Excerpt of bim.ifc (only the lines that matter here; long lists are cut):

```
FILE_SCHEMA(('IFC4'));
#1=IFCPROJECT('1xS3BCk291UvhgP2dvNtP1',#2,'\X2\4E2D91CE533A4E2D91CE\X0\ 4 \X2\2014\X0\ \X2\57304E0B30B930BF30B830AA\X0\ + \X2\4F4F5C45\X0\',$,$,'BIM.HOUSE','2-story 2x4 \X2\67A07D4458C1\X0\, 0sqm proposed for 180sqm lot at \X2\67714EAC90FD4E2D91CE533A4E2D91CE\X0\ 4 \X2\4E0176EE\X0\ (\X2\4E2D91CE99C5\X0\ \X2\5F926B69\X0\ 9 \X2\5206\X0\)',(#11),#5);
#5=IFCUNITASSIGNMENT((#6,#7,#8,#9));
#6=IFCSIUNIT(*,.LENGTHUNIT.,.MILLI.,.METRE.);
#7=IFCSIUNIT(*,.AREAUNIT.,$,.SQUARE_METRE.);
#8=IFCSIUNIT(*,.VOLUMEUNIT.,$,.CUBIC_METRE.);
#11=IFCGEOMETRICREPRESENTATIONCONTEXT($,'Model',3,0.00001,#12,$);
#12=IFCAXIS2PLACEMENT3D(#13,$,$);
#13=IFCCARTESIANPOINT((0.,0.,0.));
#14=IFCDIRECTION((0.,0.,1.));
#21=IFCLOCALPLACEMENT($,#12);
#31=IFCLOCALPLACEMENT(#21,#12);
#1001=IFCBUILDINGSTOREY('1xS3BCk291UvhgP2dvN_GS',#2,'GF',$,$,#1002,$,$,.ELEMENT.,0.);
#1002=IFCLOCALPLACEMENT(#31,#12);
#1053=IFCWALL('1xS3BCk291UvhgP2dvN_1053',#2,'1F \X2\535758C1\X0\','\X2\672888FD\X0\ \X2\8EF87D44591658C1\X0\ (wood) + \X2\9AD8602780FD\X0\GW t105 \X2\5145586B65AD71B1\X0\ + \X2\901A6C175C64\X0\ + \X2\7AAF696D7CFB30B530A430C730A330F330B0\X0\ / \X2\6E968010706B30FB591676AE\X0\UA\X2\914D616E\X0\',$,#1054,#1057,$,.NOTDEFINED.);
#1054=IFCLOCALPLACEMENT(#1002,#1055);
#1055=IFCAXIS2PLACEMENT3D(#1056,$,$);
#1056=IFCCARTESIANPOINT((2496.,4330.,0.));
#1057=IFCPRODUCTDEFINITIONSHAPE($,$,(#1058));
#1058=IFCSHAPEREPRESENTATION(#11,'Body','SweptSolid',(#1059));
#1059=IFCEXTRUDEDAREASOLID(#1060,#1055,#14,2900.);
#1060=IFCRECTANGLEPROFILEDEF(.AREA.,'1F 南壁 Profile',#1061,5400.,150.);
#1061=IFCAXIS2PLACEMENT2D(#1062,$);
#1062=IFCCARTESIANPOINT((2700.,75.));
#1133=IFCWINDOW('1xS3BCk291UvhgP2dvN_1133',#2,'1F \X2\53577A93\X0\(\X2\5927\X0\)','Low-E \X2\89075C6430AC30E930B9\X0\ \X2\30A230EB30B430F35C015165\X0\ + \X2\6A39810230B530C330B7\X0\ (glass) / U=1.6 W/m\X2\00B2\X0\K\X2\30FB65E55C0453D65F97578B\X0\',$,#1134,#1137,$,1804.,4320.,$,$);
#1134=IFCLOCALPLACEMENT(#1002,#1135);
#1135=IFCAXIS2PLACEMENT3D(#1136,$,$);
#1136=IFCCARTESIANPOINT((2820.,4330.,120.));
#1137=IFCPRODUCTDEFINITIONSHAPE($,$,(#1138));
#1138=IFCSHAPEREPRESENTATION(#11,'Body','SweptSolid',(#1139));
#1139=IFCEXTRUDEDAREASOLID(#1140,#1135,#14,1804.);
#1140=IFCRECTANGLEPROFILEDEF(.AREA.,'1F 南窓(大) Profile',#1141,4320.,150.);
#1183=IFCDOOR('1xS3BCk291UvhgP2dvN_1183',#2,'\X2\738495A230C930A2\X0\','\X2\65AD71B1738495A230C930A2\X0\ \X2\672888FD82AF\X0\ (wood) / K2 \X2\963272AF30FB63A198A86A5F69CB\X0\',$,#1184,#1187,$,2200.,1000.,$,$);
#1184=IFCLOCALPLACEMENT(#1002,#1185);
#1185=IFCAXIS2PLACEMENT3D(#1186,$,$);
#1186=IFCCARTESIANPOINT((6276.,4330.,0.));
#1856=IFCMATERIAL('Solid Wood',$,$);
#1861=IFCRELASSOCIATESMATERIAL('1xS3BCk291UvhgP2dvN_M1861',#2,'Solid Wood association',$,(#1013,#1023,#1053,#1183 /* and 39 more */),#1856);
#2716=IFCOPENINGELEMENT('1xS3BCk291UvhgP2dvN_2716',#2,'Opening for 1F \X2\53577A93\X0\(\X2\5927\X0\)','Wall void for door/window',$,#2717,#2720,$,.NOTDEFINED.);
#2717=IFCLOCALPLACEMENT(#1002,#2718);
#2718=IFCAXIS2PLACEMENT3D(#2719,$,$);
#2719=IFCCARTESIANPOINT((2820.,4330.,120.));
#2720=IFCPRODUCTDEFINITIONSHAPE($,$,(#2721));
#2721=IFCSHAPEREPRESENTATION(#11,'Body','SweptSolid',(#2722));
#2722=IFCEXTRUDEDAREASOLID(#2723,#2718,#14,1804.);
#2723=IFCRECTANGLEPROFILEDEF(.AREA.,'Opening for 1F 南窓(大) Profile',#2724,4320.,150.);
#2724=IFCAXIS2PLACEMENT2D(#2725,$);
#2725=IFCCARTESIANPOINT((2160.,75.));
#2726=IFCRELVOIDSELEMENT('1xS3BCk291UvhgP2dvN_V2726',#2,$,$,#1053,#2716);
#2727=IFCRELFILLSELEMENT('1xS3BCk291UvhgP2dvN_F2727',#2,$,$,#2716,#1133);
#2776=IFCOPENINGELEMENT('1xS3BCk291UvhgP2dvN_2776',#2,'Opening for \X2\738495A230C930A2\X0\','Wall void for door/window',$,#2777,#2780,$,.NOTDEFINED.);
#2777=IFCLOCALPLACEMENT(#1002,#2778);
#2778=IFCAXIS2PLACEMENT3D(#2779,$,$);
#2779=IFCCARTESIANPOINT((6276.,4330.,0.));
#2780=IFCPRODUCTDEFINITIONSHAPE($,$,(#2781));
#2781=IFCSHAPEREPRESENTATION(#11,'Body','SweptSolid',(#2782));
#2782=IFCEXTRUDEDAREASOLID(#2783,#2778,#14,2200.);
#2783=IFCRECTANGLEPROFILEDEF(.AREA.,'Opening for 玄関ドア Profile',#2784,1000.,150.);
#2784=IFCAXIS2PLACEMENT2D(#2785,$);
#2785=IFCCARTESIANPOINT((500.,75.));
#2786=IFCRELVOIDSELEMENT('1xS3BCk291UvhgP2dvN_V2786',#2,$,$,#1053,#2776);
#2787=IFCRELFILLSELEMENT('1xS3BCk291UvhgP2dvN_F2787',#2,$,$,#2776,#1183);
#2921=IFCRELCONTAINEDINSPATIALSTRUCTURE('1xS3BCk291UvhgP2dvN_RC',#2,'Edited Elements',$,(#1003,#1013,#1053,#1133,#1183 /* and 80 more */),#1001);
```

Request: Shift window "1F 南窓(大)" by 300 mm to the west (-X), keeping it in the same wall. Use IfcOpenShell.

```python
import ifcopenshell
import ifcopenshell.api.geometry
import ifcopenshell.util.placement
import ifcopenshell.util.unit

model = ifcopenshell.open("bim.ifc")
unit_scale = ifcopenshell.util.unit.calculate_unit_scale(model)

window = model.by_guid("1xS3BCk291UvhgP2dvN_1133")
opening = window.FillsVoids[0].RelatingOpeningElement
wall = opening.VoidsElements[0].RelatingBuildingElement

wall_matrix = ifcopenshell.util.placement.get_local_placement(wall.ObjectPlacement)
shift = wall_matrix[:3, 0] * -0.3 / unit_scale
before = ifcopenshell.util.placement.get_local_placement(window.ObjectPlacement)[:3, 3].copy()

# The window is not placed relative to its opening, so move both.
for product in (opening, window):
    matrix = ifcopenshell.util.placement.get_local_placement(product.ObjectPlacement)
    matrix[:3, 3] += shift
    ifcopenshell.api.geometry.edit_object_placement(model, product=product, matrix=matrix, is_si=False)

after = ifcopenshell.util.placement.get_local_placement(window.ObjectPlacement)[:3, 3]
print("window moved by", (after - before).round(3) + 0.0)

model.write("bim_updated.ifc")
```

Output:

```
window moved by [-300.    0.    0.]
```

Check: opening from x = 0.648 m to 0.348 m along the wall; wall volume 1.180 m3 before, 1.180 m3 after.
